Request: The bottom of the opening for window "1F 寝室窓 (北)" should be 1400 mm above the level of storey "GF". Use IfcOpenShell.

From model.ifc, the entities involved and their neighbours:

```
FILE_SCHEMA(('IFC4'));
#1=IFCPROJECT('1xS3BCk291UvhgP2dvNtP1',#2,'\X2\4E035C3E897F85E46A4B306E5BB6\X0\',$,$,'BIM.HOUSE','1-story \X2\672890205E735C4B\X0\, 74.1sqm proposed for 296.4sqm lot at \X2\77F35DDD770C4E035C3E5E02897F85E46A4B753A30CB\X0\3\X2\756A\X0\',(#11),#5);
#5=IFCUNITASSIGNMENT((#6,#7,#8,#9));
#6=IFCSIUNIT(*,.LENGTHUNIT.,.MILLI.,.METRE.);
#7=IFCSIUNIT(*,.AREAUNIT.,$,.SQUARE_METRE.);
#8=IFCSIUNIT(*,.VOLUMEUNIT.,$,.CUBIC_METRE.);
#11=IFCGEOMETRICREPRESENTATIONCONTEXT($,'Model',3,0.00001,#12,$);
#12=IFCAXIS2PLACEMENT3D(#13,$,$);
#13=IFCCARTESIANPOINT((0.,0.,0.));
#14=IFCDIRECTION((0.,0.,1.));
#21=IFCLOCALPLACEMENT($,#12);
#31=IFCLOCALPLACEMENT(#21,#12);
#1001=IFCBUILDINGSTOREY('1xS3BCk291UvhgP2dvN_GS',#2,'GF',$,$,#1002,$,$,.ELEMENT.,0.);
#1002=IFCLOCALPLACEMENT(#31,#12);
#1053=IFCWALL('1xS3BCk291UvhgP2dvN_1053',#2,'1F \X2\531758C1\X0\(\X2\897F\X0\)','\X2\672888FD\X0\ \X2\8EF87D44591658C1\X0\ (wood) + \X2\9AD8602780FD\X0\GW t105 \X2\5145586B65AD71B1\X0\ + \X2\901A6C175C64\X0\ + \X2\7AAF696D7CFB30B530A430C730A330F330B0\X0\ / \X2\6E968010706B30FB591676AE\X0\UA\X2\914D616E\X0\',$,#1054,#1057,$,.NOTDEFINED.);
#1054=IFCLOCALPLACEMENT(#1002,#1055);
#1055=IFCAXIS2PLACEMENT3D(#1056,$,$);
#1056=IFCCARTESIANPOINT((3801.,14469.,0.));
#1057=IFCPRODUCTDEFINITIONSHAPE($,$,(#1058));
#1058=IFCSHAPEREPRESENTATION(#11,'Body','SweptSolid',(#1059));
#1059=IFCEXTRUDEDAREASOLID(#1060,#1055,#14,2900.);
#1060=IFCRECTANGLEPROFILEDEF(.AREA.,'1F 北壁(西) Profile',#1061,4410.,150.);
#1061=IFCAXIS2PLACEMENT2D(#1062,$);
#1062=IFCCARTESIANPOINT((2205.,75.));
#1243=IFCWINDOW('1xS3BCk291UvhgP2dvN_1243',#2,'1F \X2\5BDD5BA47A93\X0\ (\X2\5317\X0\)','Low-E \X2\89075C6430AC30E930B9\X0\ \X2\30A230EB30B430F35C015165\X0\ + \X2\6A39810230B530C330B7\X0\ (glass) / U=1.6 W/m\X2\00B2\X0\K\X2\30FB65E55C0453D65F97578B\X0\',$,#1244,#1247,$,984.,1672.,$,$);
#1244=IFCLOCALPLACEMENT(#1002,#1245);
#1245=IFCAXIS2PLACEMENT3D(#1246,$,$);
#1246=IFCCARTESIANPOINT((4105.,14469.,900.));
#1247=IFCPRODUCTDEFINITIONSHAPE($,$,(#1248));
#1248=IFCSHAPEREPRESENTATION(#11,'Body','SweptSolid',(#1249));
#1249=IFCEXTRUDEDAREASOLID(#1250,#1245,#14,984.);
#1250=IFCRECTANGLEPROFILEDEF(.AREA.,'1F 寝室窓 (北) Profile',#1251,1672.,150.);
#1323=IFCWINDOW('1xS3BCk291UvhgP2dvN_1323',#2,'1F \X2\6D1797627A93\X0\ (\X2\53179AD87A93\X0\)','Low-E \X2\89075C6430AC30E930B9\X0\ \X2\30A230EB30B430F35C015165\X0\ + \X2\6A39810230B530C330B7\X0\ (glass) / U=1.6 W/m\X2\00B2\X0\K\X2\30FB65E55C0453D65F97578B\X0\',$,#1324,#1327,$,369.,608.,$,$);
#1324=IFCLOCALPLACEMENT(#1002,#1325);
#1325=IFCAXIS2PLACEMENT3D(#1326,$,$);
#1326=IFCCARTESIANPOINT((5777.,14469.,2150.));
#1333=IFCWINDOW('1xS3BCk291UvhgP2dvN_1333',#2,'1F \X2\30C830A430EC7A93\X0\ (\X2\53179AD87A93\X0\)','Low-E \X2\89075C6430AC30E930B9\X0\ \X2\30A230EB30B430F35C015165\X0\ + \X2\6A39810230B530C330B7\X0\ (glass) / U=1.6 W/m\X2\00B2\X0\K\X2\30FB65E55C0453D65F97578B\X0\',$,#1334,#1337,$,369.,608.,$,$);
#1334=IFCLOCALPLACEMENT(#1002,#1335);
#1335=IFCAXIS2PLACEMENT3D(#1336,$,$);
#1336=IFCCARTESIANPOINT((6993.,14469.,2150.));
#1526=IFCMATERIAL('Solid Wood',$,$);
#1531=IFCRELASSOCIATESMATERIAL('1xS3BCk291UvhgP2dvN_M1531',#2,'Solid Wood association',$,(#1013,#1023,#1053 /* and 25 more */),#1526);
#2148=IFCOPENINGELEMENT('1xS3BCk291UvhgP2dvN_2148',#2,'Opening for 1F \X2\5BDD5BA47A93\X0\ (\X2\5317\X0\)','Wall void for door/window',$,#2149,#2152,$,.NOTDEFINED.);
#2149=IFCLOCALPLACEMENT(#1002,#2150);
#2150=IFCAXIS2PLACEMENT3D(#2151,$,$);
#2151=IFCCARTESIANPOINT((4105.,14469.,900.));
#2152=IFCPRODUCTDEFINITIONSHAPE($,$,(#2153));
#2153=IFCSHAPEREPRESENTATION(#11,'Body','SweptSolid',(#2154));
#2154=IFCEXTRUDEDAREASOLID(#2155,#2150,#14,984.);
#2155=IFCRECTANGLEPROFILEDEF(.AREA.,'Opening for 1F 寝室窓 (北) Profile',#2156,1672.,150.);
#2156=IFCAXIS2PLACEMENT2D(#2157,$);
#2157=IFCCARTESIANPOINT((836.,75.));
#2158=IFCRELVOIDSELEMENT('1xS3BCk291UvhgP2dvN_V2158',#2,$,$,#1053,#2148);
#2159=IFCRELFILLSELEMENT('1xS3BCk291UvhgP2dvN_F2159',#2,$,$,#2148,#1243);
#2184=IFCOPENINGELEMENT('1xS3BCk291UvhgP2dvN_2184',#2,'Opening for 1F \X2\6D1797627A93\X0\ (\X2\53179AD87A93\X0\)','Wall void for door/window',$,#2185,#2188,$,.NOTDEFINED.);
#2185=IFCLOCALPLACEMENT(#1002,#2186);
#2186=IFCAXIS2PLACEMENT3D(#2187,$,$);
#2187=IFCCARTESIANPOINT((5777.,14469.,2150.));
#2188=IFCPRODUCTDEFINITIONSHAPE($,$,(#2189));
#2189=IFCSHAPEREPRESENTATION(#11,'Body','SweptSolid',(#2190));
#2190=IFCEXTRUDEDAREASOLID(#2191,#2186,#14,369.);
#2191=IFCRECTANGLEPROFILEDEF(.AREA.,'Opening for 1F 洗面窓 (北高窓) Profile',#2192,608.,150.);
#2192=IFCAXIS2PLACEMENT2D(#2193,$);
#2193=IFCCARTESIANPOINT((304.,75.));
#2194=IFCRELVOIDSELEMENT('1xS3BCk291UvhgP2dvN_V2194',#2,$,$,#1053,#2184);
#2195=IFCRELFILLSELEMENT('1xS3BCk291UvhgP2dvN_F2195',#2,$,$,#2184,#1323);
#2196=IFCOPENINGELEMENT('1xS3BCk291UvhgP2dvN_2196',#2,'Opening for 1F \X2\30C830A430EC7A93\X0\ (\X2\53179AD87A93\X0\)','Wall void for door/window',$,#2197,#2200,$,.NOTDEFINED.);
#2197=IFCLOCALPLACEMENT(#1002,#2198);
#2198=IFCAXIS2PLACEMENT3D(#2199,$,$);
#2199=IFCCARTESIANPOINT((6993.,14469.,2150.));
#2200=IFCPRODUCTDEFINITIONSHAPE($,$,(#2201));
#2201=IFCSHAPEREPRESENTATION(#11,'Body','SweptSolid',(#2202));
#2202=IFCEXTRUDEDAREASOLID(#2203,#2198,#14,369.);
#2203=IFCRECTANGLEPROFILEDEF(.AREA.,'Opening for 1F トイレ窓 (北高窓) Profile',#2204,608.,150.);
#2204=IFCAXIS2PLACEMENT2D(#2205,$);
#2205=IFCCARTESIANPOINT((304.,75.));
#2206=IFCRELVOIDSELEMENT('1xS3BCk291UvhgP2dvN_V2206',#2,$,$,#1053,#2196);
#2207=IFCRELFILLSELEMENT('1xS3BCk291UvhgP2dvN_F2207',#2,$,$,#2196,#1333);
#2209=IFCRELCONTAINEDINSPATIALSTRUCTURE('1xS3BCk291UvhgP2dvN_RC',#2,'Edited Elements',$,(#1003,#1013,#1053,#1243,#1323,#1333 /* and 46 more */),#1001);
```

```python
import numpy as np
import ifcopenshell
import ifcopenshell.api.geometry
import ifcopenshell.geom
import ifcopenshell.util.element
import ifcopenshell.util.placement
import ifcopenshell.util.shape
import ifcopenshell.util.unit

model = ifcopenshell.open("model.ifc")
unit_scale = ifcopenshell.util.unit.calculate_unit_scale(model)

window = model.by_guid("1xS3BCk291UvhgP2dvN_1243")
opening = window.FillsVoids[0].RelatingOpeningElement
storey = ifcopenshell.util.element.get_container(window, ifc_class="IfcBuildingStorey")
level = ifcopenshell.util.placement.get_local_placement(storey.ObjectPlacement)[2, 3]

# The opening's origin need not be at the sill, so measure its lowest point.
shape = ifcopenshell.geom.create_shape(ifcopenshell.geom.settings(), opening)
bottom = ifcopenshell.util.shape.get_shape_bottom_elevation(shape, shape.geometry) / unit_scale
dz = level + 1.4 / unit_scale - bottom

shift = np.array([0.0, 0.0, dz])
# The window is not placed relative to its opening, so move both.
for product in (opening, window):
    matrix = ifcopenshell.util.placement.get_local_placement(product.ObjectPlacement)
    matrix[:3, 3] += shift
    ifcopenshell.api.geometry.edit_object_placement(model, product=product, matrix=matrix, is_si=False)

print(f"moved by {dz * unit_scale:+.3f} m")

model.write("model-out.ifc")
```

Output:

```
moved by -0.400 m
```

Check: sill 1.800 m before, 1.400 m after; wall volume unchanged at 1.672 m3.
